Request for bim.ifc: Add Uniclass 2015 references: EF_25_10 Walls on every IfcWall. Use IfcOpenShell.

First a look at what the model holds.

```python
import ifcopenshell

model = ifcopenshell.open("bim.ifc")
print(model.schema)
print("classifications:", [c.Name for c in model.by_type("IfcClassification")])
for ifc_class in ("IfcDoor", "IfcRoof", "IfcStair", "IfcWall", "IfcWindow"):
    print(ifc_class, len(model.by_type(ifc_class)))
```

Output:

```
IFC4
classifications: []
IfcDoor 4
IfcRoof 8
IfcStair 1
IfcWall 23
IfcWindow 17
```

```python
import ifcopenshell
import ifcopenshell.api.classification

model = ifcopenshell.open("bim.ifc")

system = ifcopenshell.api.classification.add_classification(model, classification="Uniclass 2015")

codes = {
    "IfcWall": ("EF_25_10", "Walls"),
}
for ifc_class, (code, name) in codes.items():
    products = model.by_type(ifc_class)
    ifcopenshell.api.classification.add_reference(
        model, products=products, classification=system, identification=code, name=name
    )
    print(code, len(products))

model.write("bim_rev.ifc")
```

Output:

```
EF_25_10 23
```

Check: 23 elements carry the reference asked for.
